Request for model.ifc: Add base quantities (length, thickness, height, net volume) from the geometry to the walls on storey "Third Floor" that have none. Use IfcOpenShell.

First a look at what the model holds.

```python
import ifcopenshell
import ifcopenshell.util.element
import ifcopenshell.util.unit

model = ifcopenshell.open("model.ifc")
print(model.schema)
for unit_type in ("LENGTHUNIT", "AREAUNIT", "VOLUMEUNIT"):
    print(unit_type, ifcopenshell.util.unit.calculate_unit_scale(model, unit_type))
storey = next(s for s in model.by_type("IfcBuildingStorey") if s.Name == "Third Floor")
walls = [e for e in ifcopenshell.util.element.get_decomposition(storey) if e.is_a("IfcWall")]
for e in sorted(walls, key=lambda e: e.id()):
    print(e.id(), e.is_a(), e.Name, list(ifcopenshell.util.element.get_psets(e, qtos_only=True)), sep=" | ")
```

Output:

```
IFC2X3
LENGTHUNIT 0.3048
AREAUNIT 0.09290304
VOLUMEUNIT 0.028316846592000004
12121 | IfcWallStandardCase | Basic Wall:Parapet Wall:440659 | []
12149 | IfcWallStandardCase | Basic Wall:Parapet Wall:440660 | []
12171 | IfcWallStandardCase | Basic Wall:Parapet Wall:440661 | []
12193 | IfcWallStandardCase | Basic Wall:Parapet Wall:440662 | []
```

```python
import ifcopenshell
import ifcopenshell.api.pset
import ifcopenshell.geom
import ifcopenshell.util.element
import ifcopenshell.util.shape
import ifcopenshell.util.unit

model = ifcopenshell.open("model.ifc")
unit_scale = ifcopenshell.util.unit.calculate_unit_scale(model)
volume_scale = ifcopenshell.util.unit.calculate_unit_scale(model, "VOLUMEUNIT")
settings = ifcopenshell.geom.settings()

storey = next(s for s in model.by_type("IfcBuildingStorey") if s.Name == "Third Floor")
walls = [e for e in ifcopenshell.util.element.get_decomposition(storey) if e.is_a("IfcWall")]

for e in sorted(walls, key=lambda e: e.id()):
    if ifcopenshell.util.element.get_psets(e, qtos_only=True, should_inherit=False):
        continue
    # Geometry comes back in metres, in the element's own axes.
    shape = ifcopenshell.geom.create_shape(settings, e)
    values = {
        "Length": ifcopenshell.util.shape.get_x(shape.geometry) / unit_scale,
        "Width": ifcopenshell.util.shape.get_y(shape.geometry) / unit_scale,
        "Height": ifcopenshell.util.shape.get_z(shape.geometry) / unit_scale,
        "NetVolume": ifcopenshell.util.shape.get_volume(shape.geometry) / volume_scale,
    }
    qto = ifcopenshell.api.pset.add_qto(model, product=e, name="BaseQuantities")
    ifcopenshell.api.pset.edit_qto(model, qto=qto, properties=values)
    print(e.id(), {k: round(v, 3) for k, v in values.items()})

model.write("model-out.ifc")
```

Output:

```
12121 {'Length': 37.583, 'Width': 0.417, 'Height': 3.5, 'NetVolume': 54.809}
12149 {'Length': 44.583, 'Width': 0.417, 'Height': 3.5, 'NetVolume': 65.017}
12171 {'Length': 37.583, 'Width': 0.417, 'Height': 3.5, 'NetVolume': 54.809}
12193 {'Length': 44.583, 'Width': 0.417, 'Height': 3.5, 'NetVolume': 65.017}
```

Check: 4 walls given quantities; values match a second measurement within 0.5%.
